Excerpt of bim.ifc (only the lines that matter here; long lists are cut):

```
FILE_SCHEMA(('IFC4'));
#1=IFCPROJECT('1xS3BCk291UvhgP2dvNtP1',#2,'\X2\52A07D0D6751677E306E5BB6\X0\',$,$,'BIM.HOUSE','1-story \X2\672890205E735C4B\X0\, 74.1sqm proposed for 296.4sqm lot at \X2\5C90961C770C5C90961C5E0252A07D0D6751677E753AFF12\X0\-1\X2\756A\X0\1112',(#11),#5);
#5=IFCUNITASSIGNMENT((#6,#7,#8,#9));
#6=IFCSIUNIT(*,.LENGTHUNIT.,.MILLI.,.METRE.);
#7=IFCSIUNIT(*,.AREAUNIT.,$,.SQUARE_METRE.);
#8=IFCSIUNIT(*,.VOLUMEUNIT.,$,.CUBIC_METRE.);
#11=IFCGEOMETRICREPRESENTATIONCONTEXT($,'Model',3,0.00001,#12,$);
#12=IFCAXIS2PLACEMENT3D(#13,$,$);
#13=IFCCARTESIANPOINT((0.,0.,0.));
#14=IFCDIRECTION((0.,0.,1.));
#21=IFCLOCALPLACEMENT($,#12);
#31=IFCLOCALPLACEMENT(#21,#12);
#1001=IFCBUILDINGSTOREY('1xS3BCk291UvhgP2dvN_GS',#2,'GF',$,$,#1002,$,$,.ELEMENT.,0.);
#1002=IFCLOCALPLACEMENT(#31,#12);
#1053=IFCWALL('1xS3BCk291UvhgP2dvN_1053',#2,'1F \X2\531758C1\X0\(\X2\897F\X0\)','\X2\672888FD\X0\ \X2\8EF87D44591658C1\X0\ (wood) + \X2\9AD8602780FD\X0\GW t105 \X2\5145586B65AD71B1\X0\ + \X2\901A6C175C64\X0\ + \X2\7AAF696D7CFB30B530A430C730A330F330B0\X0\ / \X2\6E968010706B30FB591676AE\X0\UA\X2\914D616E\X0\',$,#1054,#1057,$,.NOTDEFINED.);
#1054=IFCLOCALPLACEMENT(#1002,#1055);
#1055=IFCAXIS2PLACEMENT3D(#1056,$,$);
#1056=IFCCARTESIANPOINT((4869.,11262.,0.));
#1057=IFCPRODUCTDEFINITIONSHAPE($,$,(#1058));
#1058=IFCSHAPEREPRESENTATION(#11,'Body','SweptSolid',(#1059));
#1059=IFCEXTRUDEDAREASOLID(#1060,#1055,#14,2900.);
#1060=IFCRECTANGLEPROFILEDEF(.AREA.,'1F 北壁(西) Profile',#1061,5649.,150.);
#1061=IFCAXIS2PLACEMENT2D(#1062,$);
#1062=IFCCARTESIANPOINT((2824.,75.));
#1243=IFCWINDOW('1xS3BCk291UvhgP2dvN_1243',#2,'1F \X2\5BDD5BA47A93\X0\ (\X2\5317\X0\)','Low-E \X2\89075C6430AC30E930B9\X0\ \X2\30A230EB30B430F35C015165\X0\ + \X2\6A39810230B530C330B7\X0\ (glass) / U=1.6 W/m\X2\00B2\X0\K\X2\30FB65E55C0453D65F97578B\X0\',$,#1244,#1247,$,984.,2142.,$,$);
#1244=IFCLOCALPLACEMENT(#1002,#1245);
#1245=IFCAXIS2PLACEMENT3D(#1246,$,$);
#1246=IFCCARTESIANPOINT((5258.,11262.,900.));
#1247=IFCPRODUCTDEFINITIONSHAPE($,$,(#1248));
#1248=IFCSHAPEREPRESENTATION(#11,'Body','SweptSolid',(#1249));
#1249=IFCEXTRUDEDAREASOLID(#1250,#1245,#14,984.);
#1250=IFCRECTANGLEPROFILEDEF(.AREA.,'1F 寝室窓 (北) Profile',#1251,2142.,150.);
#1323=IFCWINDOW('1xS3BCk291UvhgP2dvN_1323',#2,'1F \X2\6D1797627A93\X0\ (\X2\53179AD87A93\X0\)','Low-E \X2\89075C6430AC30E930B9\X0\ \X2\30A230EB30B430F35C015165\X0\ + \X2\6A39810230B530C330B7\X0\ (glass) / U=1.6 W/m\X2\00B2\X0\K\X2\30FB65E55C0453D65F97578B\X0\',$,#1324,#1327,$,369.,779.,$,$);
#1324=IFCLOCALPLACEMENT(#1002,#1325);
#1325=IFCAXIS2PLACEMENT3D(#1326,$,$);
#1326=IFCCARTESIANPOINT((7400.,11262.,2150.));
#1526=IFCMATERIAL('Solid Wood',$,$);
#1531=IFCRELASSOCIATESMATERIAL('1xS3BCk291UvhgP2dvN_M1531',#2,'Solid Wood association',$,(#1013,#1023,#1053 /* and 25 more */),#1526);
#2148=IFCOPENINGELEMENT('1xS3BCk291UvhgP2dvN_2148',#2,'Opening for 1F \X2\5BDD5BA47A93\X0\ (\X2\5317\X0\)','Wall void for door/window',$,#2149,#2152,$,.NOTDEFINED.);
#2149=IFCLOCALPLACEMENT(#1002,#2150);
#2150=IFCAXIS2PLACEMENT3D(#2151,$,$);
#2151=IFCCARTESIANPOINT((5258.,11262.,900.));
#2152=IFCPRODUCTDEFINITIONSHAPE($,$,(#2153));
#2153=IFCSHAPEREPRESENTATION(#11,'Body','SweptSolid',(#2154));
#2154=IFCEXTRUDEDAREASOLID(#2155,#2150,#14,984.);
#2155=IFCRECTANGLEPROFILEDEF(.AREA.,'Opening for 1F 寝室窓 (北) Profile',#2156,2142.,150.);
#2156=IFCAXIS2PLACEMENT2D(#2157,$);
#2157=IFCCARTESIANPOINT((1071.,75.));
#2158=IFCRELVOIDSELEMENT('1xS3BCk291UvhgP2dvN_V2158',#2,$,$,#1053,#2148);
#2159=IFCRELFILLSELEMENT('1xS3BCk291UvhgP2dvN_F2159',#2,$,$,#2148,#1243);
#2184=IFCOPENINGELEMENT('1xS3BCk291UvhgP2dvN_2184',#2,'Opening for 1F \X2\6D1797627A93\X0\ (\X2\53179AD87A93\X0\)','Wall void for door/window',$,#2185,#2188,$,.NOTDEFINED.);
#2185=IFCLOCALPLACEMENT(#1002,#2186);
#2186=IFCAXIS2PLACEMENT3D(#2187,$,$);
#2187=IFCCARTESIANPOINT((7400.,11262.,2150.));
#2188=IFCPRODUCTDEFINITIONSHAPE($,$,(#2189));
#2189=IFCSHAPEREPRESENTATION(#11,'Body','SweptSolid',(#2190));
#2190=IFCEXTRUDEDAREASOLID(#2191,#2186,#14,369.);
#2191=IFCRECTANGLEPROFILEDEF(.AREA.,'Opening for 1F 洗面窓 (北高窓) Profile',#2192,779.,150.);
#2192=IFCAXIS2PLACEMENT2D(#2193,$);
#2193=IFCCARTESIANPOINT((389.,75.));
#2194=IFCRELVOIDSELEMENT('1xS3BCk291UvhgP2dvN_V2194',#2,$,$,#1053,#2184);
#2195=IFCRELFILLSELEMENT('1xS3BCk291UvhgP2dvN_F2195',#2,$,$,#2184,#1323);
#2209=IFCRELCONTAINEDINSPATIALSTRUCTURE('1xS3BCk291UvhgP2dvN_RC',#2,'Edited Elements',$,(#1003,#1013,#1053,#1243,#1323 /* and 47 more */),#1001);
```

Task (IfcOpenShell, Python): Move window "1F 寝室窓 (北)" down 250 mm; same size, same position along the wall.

```python
import numpy as np
import ifcopenshell
import ifcopenshell.api.geometry
import ifcopenshell.util.placement
import ifcopenshell.util.unit

model = ifcopenshell.open("bim.ifc")
unit_scale = ifcopenshell.util.unit.calculate_unit_scale(model)

window = model.by_guid("1xS3BCk291UvhgP2dvN_1243")
opening = window.FillsVoids[0].RelatingOpeningElement
dz = -250.0

shift = np.array([0.0, 0.0, dz])
# The window is not placed relative to its opening, so move both.
for product in (opening, window):
    matrix = ifcopenshell.util.placement.get_local_placement(product.ObjectPlacement)
    matrix[:3, 3] += shift
    ifcopenshell.api.geometry.edit_object_placement(model, product=product, matrix=matrix, is_si=False)

print(f"moved by {dz * unit_scale:+.3f} m")

model.write("bim_rev.ifc")
```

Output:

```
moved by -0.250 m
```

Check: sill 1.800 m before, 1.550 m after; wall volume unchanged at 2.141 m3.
